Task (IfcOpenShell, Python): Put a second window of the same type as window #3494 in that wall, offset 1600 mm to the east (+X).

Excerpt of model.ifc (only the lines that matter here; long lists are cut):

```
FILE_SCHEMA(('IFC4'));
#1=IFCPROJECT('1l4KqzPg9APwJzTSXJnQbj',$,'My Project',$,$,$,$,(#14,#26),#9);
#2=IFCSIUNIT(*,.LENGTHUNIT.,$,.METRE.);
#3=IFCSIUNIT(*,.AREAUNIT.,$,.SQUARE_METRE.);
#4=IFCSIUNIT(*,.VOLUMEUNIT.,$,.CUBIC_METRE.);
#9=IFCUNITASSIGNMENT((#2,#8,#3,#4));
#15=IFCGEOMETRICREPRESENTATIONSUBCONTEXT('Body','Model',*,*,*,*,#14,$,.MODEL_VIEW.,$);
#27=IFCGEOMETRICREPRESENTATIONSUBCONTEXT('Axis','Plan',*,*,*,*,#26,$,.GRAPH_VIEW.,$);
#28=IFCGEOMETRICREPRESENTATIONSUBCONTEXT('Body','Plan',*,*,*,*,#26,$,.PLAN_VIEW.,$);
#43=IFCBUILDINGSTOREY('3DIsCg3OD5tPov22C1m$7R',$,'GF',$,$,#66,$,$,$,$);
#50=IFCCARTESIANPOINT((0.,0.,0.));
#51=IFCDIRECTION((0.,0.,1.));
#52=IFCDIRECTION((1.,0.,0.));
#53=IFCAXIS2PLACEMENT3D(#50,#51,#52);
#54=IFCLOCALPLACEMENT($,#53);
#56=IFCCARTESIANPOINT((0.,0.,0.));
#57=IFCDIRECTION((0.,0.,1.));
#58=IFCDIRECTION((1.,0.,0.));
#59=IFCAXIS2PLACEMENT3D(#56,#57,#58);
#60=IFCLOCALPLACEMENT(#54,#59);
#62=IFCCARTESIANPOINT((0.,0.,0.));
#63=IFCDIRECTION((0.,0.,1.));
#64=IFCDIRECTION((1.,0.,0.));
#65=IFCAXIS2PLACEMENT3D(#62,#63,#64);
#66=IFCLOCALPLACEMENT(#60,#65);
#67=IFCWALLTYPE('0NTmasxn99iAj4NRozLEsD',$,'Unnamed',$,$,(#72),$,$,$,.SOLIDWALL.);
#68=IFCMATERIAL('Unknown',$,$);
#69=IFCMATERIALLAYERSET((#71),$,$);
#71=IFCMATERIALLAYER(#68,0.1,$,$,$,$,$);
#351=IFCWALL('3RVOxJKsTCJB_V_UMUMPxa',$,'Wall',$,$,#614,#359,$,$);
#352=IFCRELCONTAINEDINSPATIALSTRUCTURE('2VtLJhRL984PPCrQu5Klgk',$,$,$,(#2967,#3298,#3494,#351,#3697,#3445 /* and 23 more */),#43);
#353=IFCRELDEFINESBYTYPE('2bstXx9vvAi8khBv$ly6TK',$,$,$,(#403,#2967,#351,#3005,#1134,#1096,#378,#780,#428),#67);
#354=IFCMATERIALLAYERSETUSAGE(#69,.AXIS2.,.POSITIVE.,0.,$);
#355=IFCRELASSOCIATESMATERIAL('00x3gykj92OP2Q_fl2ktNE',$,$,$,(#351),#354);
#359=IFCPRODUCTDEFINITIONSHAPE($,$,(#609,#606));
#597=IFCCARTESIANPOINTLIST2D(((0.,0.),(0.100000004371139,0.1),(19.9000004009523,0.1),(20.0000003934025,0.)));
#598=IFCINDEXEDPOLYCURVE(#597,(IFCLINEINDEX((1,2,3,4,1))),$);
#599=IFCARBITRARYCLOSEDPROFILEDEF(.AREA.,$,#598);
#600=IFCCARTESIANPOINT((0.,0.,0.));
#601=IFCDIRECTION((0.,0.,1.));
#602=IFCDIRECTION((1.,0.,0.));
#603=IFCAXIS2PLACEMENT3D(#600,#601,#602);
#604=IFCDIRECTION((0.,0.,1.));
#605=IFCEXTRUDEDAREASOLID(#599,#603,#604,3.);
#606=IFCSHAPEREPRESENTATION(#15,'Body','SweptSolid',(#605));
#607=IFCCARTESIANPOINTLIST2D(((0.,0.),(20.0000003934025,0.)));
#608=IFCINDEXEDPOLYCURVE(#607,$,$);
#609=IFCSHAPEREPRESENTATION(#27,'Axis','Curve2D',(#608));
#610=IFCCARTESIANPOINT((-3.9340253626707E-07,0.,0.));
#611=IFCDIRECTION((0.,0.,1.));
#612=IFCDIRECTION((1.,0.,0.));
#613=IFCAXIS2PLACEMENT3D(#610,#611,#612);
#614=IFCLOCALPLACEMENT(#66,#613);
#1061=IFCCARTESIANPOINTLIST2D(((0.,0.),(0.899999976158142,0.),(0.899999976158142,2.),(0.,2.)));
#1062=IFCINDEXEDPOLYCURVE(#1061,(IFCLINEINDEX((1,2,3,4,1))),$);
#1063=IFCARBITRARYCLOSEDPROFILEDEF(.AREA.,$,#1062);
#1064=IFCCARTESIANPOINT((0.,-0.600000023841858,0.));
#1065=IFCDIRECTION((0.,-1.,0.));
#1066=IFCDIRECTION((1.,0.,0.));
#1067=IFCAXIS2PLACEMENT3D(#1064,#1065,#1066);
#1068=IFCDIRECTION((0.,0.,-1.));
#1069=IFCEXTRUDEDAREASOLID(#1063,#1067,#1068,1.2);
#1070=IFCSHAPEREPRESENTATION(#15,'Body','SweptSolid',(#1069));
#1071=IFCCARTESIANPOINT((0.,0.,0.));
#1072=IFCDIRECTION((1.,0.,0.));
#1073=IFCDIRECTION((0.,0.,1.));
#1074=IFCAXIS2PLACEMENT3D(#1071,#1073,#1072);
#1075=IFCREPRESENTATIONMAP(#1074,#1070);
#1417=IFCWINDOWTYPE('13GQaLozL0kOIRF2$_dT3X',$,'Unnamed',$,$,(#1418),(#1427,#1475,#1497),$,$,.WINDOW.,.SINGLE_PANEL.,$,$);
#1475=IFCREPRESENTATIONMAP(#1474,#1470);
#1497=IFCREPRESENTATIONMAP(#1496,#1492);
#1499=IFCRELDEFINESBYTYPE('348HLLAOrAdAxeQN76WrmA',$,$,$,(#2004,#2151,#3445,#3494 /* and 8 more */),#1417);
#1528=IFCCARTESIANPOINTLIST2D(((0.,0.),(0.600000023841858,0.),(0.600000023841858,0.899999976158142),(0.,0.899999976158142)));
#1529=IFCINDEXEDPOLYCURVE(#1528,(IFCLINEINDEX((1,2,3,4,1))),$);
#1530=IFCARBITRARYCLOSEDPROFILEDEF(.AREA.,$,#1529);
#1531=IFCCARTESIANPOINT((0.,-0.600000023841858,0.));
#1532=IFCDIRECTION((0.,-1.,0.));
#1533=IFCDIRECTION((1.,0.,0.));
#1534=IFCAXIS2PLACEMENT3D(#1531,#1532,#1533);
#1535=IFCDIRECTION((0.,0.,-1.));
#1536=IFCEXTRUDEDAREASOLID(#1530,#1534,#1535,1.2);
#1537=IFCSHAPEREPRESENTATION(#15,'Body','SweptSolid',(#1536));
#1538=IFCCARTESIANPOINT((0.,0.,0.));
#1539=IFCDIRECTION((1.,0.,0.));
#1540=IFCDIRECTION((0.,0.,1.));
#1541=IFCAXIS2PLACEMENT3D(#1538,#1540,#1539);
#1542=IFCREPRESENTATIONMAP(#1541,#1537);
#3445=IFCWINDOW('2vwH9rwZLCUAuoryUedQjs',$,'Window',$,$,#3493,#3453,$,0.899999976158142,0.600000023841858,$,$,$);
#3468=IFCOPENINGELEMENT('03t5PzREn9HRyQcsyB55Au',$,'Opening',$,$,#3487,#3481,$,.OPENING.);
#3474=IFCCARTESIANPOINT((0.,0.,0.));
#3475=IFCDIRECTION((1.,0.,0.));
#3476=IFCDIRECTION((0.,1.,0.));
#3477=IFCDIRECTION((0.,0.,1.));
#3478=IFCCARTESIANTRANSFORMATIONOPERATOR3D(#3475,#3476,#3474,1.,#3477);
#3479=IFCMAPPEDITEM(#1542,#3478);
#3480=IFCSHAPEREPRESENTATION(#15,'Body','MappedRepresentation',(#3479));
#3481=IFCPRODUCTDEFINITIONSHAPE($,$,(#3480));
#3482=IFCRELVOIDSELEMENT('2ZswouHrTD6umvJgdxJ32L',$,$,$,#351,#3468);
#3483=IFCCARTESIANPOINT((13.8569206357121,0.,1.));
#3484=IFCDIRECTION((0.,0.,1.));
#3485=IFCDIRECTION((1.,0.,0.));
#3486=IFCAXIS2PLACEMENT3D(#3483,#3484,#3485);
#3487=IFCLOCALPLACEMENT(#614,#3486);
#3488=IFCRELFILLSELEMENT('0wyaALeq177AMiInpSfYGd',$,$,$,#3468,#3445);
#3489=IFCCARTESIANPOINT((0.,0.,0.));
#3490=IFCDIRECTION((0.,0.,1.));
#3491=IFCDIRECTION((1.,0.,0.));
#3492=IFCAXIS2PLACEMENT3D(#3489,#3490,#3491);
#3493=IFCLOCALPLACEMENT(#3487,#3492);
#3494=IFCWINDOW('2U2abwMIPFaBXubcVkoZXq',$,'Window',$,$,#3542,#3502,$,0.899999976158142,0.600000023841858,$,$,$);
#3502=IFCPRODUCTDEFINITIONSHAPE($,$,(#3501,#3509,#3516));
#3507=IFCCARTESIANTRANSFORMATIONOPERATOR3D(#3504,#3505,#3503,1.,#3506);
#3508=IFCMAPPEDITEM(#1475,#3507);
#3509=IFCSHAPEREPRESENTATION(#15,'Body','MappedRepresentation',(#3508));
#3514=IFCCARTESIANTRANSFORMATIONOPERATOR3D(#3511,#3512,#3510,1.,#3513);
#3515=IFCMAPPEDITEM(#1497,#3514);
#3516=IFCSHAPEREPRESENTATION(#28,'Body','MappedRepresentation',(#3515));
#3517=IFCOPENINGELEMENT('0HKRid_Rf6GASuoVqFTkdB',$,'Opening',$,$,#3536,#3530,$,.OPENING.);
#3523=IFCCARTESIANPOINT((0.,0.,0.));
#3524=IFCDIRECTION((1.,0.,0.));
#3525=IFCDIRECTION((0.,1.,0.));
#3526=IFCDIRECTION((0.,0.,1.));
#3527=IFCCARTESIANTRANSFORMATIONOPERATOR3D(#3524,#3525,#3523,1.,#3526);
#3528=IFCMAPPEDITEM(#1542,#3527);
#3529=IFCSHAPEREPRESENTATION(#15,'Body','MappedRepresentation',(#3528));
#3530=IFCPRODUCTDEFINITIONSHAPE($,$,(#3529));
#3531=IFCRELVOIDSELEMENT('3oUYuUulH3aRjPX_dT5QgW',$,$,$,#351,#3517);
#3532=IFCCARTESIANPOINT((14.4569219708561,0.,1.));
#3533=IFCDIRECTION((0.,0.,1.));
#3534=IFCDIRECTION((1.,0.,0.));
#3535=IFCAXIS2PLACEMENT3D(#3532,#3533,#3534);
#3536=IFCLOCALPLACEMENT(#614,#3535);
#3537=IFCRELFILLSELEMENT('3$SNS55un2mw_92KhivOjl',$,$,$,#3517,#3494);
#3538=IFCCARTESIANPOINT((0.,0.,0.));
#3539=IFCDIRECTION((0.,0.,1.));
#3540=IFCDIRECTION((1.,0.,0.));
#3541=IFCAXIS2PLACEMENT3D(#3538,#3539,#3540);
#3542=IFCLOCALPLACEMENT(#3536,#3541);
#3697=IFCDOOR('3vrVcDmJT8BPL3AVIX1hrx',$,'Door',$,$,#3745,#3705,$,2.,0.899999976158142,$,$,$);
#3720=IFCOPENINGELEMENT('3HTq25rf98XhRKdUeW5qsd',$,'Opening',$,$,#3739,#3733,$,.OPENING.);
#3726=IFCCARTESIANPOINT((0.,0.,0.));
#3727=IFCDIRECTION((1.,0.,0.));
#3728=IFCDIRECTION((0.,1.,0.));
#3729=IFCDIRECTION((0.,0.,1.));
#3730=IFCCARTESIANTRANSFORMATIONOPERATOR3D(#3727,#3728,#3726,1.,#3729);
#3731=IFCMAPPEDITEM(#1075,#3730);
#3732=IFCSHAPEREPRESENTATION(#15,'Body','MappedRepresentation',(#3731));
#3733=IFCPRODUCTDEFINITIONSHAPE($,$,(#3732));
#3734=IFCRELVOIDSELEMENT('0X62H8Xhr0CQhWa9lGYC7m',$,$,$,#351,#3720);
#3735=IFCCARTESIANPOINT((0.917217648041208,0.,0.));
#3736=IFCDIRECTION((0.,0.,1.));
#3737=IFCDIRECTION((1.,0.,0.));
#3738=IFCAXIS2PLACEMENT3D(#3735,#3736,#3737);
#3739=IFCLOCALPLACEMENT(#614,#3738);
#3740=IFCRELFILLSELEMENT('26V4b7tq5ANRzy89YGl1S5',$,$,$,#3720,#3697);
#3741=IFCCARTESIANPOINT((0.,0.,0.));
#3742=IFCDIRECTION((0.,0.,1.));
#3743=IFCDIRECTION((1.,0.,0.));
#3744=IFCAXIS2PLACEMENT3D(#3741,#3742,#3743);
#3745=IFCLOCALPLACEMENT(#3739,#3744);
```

```python
import ifcopenshell
import ifcopenshell.api.feature
import ifcopenshell.api.geometry
import ifcopenshell.api.root
import ifcopenshell.geom
import ifcopenshell.util.element
import ifcopenshell.util.placement
import ifcopenshell.util.shape

model = ifcopenshell.open("model.ifc")
settings = ifcopenshell.geom.settings()


def volume(element):
    """Net volume in cubic metres, openings subtracted."""
    shape = ifcopenshell.geom.create_shape(settings, element)
    return ifcopenshell.util.shape.get_volume(shape.geometry)


window = model.by_guid("2U2abwMIPFaBXubcVkoZXq")
opening = window.FillsVoids[0].RelatingOpeningElement
wall = opening.VoidsElements[0].RelatingBuildingElement
before = volume(wall)
shift = ifcopenshell.util.placement.get_local_placement(wall.ObjectPlacement)[:3, 0] * 1.6

# copy_class copies the void relationship, type, container and properties, but no geometry.
new_opening = ifcopenshell.api.root.copy_class(model, product=opening)
new_opening.Representation = ifcopenshell.util.element.copy_deep(
    model, opening.Representation, exclude=["IfcGeometricRepresentationContext", "IfcRepresentationMap"]
)
new_window = ifcopenshell.api.root.copy_class(model, product=window)
new_window.Representation = ifcopenshell.util.element.copy_deep(
    model, window.Representation, exclude=["IfcGeometricRepresentationContext", "IfcRepresentationMap"]
)
ifcopenshell.api.feature.add_filling(model, opening=new_opening, element=new_window)

for old, new in ((opening, new_opening), (window, new_window)):
    matrix = ifcopenshell.util.placement.get_local_placement(old.ObjectPlacement)
    matrix[:3, 3] += shift
    ifcopenshell.api.geometry.edit_object_placement(model, product=new, matrix=matrix, is_si=False)

after = volume(wall)

print(f"wall volume {before:.3f} -> {after:.3f} m3")

model.write("model-out.ifc")
```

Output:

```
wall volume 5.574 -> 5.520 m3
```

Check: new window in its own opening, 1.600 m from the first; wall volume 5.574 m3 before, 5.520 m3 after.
